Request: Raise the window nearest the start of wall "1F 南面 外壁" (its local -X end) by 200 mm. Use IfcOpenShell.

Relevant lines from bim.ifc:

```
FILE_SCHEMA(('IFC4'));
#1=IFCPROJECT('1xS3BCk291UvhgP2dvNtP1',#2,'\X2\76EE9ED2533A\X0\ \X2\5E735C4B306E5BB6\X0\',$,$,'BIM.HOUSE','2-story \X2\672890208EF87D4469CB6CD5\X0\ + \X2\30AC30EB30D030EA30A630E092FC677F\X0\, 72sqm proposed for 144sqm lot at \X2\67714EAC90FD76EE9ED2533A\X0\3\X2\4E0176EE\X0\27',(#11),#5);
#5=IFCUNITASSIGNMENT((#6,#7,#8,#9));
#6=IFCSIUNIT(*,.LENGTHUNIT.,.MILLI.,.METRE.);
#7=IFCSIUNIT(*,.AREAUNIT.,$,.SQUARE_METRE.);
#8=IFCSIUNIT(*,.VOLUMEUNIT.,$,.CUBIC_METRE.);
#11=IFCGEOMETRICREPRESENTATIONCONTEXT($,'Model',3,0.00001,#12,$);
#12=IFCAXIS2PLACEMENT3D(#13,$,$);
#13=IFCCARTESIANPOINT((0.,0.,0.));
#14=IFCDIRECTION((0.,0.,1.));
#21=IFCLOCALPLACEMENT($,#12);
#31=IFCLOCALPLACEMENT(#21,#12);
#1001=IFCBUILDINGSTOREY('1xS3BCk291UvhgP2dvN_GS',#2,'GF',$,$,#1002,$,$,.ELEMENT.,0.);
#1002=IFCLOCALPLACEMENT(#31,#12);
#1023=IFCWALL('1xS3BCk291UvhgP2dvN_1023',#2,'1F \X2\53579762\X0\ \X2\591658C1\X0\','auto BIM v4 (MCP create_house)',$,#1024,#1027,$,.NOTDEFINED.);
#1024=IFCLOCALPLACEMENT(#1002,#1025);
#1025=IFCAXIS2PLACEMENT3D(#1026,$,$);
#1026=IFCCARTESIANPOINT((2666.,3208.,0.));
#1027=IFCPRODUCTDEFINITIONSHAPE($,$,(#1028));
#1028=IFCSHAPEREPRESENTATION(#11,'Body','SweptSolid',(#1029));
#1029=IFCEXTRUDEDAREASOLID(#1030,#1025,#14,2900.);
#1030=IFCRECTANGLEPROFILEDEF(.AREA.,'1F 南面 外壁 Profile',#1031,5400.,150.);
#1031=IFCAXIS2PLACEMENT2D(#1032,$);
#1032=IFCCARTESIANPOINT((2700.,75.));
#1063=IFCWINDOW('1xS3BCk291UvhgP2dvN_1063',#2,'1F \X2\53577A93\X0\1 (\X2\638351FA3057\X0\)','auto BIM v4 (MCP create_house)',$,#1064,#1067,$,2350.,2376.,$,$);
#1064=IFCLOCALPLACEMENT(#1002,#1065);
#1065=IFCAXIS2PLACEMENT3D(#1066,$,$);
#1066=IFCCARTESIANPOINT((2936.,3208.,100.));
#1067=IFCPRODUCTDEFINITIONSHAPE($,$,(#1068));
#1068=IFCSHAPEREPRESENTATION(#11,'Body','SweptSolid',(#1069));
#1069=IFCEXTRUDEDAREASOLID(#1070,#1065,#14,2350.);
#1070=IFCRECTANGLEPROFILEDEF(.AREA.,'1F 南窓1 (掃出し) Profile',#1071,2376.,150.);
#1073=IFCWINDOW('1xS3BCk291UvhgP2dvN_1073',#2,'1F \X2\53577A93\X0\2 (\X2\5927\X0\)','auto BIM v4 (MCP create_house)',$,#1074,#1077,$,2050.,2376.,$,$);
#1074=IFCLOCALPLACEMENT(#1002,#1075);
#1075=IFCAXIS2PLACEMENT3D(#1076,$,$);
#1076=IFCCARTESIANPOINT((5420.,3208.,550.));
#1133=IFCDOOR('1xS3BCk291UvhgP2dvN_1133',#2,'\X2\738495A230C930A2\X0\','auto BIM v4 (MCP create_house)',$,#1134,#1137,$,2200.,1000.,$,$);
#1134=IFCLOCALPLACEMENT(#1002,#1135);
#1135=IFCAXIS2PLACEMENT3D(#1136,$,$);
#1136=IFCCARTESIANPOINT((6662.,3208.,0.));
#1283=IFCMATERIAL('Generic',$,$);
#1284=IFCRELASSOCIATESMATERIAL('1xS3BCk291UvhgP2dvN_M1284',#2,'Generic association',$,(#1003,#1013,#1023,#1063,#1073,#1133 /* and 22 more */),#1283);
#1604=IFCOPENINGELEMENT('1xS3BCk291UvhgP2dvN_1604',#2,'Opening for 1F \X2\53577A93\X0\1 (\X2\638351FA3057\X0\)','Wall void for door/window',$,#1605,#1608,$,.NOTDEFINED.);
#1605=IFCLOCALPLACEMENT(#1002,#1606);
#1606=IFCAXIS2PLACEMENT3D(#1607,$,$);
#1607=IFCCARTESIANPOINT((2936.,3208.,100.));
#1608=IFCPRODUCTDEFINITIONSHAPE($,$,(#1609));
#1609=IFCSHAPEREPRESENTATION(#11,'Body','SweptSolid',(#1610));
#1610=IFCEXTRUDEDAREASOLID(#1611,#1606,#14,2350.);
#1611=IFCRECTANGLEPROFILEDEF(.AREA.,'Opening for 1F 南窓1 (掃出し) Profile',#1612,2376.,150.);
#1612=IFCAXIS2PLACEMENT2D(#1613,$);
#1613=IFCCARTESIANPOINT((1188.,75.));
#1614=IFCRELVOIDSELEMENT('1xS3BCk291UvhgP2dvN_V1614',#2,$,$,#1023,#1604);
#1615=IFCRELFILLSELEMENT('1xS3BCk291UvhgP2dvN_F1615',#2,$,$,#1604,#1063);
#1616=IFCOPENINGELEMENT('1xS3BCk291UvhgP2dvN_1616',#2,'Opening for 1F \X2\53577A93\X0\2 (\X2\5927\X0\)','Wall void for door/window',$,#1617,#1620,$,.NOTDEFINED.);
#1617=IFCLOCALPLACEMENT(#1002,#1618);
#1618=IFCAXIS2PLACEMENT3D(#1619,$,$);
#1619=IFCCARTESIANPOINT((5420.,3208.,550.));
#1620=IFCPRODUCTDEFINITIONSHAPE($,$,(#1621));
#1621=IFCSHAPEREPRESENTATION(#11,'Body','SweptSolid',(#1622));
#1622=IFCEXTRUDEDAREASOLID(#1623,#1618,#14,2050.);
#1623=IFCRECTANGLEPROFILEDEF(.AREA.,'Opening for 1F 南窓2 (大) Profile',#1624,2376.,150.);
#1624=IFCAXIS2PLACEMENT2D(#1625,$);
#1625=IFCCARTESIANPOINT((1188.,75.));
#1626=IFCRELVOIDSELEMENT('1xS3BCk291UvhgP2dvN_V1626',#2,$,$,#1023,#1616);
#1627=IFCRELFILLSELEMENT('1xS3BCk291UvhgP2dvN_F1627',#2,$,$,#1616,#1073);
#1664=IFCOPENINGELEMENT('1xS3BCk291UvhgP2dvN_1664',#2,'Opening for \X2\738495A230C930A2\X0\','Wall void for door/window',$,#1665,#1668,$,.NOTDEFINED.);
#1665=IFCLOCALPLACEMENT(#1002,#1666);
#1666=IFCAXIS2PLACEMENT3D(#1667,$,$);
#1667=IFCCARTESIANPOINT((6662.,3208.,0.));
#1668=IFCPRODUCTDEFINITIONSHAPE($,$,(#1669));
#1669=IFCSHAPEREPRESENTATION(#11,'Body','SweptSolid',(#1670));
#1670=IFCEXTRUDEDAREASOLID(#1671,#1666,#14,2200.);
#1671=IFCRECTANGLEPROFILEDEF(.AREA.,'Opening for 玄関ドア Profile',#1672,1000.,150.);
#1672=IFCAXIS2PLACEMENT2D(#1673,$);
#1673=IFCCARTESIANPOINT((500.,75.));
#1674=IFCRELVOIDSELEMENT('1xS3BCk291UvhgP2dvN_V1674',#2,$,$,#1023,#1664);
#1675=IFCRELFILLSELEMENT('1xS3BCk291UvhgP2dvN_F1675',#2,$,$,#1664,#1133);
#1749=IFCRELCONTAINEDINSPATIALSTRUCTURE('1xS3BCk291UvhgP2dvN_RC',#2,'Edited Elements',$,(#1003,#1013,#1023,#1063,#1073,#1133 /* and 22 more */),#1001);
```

```python
import numpy as np
import ifcopenshell
import ifcopenshell.api.geometry
import ifcopenshell.util.placement
import ifcopenshell.util.unit

model = ifcopenshell.open("bim.ifc")
unit_scale = ifcopenshell.util.unit.calculate_unit_scale(model)

window = model.by_guid("1xS3BCk291UvhgP2dvN_1063")
opening = window.FillsVoids[0].RelatingOpeningElement
dz = 200.0

shift = np.array([0.0, 0.0, dz])
# The window is not placed relative to its opening, so move both.
for product in (opening, window):
    matrix = ifcopenshell.util.placement.get_local_placement(product.ObjectPlacement)
    matrix[:3, 3] += shift
    ifcopenshell.api.geometry.edit_object_placement(model, product=product, matrix=matrix, is_si=False)

print(f"moved by {dz * unit_scale:+.3f} m")

model.write("bim_edited.ifc")
```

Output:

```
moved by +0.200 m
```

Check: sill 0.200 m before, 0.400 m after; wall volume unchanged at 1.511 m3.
